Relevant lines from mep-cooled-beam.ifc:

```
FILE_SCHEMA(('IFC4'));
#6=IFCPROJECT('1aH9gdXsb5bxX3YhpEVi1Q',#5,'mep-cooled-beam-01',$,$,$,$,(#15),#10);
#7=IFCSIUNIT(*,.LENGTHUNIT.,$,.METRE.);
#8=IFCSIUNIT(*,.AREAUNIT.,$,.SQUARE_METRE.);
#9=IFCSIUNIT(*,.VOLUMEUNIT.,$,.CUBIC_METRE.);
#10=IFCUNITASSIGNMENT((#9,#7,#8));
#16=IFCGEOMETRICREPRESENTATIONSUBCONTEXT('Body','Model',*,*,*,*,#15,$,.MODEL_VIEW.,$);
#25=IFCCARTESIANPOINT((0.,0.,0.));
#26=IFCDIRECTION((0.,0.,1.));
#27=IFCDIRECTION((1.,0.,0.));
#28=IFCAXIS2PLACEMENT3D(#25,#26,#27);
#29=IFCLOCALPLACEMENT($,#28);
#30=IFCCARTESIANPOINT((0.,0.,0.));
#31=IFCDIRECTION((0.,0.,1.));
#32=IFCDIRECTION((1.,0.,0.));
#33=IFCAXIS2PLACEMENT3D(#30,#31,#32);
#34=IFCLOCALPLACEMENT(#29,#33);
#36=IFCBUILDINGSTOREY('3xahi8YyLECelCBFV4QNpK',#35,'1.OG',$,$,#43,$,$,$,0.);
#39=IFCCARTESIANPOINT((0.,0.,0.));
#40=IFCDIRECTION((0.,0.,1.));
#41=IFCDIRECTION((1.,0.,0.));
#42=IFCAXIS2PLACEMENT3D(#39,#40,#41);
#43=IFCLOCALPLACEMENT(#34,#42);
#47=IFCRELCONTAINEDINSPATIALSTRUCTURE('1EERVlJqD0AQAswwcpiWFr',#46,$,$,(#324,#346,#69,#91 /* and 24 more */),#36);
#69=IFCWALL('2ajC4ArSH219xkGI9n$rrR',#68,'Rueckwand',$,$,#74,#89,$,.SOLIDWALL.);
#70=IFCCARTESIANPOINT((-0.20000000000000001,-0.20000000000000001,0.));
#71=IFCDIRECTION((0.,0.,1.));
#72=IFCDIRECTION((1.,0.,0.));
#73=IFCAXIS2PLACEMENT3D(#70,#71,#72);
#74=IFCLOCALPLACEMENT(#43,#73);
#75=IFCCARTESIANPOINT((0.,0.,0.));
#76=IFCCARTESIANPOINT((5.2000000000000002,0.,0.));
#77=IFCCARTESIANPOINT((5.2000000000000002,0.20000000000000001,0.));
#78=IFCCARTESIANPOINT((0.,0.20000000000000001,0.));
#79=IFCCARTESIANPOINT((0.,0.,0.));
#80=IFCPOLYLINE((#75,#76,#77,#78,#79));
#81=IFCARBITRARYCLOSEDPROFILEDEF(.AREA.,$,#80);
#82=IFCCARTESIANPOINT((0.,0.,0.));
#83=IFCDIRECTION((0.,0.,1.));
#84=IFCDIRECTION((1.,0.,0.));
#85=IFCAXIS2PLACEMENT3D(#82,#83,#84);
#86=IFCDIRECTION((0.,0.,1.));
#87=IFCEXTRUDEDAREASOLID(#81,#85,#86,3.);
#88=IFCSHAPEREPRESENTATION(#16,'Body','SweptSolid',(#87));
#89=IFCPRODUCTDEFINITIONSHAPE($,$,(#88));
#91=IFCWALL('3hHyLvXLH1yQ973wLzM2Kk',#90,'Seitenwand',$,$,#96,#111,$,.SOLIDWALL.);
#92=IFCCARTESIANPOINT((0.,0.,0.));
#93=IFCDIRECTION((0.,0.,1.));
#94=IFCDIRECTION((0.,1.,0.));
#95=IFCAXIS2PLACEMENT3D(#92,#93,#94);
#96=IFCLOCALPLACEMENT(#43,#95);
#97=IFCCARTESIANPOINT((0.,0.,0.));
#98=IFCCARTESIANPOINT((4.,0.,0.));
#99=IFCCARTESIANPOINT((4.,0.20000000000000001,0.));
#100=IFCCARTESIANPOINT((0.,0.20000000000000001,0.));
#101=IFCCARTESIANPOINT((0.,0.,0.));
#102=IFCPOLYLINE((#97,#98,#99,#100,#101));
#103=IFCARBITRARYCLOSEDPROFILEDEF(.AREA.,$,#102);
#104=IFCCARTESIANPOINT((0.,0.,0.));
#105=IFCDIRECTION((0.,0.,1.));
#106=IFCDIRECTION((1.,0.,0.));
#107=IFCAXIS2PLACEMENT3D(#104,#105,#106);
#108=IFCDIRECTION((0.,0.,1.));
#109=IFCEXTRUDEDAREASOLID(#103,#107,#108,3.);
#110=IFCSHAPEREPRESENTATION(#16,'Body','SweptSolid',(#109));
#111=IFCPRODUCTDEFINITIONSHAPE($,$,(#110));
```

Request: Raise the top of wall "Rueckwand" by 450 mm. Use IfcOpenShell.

```python
import ifcopenshell
import ifcopenshell.geom
import ifcopenshell.util.representation
import ifcopenshell.util.shape
import ifcopenshell.util.unit

model = ifcopenshell.open("mep-cooled-beam.ifc")
unit_scale = ifcopenshell.util.unit.calculate_unit_scale(model)
settings = ifcopenshell.geom.settings()


def volume(element):
    """Net volume in cubic metres, openings subtracted."""
    shape = ifcopenshell.geom.create_shape(settings, element)
    return ifcopenshell.util.shape.get_volume(shape.geometry)


wall = model.by_guid("2ajC4ArSH219xkGI9n$rrR")
before = volume(wall)

body = ifcopenshell.util.representation.get_representation(wall, "Model", "Body")
solid = body.Items[0]
old_height = solid.Depth
solid.Depth += 0.45 / unit_scale
after = volume(wall)

print(f"height {old_height:g} -> {solid.Depth:g}, volume {before:.3f} -> {after:.3f} m3")

model.write("mep-cooled-beam_rev.ifc")
```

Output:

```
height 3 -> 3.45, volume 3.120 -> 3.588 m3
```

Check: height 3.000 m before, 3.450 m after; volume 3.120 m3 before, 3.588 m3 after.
